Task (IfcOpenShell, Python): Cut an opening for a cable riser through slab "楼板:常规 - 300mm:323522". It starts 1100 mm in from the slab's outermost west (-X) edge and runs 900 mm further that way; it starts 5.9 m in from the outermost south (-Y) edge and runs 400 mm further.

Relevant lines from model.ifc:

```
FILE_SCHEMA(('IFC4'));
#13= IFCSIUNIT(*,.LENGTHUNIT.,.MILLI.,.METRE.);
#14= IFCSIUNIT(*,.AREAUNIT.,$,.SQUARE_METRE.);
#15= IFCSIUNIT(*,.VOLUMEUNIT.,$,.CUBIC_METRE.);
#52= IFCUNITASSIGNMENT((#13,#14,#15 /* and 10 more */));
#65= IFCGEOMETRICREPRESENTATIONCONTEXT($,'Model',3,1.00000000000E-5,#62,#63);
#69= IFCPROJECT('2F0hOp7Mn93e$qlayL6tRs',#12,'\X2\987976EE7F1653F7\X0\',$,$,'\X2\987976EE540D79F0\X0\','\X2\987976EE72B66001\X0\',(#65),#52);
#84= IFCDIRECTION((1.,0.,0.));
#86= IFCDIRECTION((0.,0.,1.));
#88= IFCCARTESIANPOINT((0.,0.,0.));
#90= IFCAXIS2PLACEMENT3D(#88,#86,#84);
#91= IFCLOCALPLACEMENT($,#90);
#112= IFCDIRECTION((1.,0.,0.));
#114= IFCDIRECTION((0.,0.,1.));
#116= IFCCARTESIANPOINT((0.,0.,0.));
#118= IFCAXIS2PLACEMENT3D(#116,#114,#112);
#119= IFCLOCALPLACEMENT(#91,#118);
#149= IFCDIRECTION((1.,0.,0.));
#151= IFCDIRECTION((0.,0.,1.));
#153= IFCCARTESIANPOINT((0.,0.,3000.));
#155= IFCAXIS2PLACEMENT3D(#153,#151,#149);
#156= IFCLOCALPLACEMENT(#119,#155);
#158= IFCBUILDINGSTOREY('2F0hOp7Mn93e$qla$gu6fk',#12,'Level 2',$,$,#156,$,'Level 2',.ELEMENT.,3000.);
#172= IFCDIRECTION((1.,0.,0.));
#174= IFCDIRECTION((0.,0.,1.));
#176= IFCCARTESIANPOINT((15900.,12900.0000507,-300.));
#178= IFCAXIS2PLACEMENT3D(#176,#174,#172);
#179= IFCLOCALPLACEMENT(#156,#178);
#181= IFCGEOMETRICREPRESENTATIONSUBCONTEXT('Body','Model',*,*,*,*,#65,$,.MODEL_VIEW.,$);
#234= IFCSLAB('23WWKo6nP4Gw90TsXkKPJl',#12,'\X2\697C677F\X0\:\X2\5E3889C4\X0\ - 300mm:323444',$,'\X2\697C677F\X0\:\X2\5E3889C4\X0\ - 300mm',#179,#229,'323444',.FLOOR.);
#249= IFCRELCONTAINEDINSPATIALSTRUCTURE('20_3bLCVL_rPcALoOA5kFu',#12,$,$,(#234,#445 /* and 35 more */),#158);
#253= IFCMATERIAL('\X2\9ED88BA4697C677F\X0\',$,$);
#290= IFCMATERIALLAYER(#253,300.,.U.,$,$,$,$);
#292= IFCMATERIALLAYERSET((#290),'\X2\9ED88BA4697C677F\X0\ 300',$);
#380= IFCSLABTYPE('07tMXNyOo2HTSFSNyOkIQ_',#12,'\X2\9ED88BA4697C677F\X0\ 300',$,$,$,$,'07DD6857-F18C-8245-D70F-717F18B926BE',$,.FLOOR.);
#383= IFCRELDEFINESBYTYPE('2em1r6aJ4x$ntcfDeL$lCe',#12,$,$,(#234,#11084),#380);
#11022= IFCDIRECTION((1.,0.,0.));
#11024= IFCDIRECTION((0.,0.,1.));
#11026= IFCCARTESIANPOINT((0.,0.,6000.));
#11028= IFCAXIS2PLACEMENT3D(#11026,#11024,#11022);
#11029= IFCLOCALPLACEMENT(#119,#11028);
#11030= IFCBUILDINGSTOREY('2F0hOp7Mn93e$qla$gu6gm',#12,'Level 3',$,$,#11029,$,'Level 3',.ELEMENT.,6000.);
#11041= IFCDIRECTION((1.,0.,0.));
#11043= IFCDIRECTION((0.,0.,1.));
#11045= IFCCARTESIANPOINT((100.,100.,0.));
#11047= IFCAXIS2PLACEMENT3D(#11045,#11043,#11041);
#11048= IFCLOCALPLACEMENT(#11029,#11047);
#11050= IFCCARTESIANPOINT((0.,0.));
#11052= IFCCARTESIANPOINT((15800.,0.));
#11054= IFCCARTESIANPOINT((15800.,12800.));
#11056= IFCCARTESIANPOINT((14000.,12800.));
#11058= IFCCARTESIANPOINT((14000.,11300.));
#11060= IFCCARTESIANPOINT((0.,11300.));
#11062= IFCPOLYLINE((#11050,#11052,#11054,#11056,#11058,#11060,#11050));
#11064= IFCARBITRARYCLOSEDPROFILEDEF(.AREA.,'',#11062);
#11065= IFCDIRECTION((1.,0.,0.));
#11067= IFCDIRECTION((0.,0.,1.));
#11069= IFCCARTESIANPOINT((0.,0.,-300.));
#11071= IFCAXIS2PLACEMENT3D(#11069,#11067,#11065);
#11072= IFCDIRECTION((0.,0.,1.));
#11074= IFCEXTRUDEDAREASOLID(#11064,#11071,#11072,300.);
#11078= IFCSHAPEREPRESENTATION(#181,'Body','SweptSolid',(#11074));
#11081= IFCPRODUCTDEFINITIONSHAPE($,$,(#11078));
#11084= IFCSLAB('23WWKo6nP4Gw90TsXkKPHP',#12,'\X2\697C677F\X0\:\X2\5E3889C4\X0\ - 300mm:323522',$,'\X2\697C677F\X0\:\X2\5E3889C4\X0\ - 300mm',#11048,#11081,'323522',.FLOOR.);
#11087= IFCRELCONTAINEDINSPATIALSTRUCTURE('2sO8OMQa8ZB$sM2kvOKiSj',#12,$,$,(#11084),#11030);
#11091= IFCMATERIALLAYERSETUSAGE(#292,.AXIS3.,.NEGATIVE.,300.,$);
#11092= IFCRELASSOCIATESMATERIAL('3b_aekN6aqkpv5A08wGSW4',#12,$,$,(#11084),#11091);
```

```python
import numpy as np
import ifcopenshell
import ifcopenshell.api.feature
import ifcopenshell.api.geometry
import ifcopenshell.api.root
import ifcopenshell.geom
import ifcopenshell.util.placement
import ifcopenshell.util.representation
import ifcopenshell.util.shape
import ifcopenshell.util.unit

model = ifcopenshell.open("model.ifc")
unit_scale = ifcopenshell.util.unit.calculate_unit_scale(model)
settings = ifcopenshell.geom.settings()


def volume(element):
    """Net volume in cubic metres, openings subtracted."""
    shape = ifcopenshell.geom.create_shape(settings, element)
    return ifcopenshell.util.shape.get_volume(shape.geometry)


slab = model.by_guid("23WWKo6nP4Gw90TsXkKPHP")
before = volume(slab)

# Extent in the slab's own axes, in metres. The edges named are its -X and -Y sides.
slab_shape = ifcopenshell.geom.create_shape(settings, slab)
vertices = ifcopenshell.util.shape.get_vertices(slab_shape.geometry)
x_min, y_min, bottom = vertices.min(axis=0)
top = vertices[:, 2].max()

opening = ifcopenshell.api.root.create_entity(model, ifc_class="IfcOpeningElement", name="Cable riser opening", predefined_type="OPENING")
context = ifcopenshell.util.representation.get_context(model, "Model", "Body", "MODEL_VIEW")
width, depth = 0.9, 0.4
outline = [(0.0, 0.0), (width, 0.0), (width, depth), (0.0, depth), (0.0, 0.0)]
# Overshoot both faces by 50 mm so the cut is clean.
shape = ifcopenshell.api.geometry.add_slab_representation(
    model, context=context, depth=top - bottom + 0.1, polyline=outline
)
ifcopenshell.api.geometry.assign_representation(model, product=opening, representation=shape)

matrix = ifcopenshell.util.placement.get_local_placement(slab.ObjectPlacement)
matrix[:, 3] = matrix @ np.append(np.array([x_min + 1.1, y_min + 5.9, bottom - 0.05]) / unit_scale, 1.0)
ifcopenshell.api.geometry.edit_object_placement(model, product=opening, matrix=matrix, is_si=False)
ifcopenshell.api.feature.add_feature(model, feature=opening, element=slab)

after = volume(slab)

print(f"slab volume {before:.3f} -> {after:.3f} m3")

model.write("model-out.ifc")
```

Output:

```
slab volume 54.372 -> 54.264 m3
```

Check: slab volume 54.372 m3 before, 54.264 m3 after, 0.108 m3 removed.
